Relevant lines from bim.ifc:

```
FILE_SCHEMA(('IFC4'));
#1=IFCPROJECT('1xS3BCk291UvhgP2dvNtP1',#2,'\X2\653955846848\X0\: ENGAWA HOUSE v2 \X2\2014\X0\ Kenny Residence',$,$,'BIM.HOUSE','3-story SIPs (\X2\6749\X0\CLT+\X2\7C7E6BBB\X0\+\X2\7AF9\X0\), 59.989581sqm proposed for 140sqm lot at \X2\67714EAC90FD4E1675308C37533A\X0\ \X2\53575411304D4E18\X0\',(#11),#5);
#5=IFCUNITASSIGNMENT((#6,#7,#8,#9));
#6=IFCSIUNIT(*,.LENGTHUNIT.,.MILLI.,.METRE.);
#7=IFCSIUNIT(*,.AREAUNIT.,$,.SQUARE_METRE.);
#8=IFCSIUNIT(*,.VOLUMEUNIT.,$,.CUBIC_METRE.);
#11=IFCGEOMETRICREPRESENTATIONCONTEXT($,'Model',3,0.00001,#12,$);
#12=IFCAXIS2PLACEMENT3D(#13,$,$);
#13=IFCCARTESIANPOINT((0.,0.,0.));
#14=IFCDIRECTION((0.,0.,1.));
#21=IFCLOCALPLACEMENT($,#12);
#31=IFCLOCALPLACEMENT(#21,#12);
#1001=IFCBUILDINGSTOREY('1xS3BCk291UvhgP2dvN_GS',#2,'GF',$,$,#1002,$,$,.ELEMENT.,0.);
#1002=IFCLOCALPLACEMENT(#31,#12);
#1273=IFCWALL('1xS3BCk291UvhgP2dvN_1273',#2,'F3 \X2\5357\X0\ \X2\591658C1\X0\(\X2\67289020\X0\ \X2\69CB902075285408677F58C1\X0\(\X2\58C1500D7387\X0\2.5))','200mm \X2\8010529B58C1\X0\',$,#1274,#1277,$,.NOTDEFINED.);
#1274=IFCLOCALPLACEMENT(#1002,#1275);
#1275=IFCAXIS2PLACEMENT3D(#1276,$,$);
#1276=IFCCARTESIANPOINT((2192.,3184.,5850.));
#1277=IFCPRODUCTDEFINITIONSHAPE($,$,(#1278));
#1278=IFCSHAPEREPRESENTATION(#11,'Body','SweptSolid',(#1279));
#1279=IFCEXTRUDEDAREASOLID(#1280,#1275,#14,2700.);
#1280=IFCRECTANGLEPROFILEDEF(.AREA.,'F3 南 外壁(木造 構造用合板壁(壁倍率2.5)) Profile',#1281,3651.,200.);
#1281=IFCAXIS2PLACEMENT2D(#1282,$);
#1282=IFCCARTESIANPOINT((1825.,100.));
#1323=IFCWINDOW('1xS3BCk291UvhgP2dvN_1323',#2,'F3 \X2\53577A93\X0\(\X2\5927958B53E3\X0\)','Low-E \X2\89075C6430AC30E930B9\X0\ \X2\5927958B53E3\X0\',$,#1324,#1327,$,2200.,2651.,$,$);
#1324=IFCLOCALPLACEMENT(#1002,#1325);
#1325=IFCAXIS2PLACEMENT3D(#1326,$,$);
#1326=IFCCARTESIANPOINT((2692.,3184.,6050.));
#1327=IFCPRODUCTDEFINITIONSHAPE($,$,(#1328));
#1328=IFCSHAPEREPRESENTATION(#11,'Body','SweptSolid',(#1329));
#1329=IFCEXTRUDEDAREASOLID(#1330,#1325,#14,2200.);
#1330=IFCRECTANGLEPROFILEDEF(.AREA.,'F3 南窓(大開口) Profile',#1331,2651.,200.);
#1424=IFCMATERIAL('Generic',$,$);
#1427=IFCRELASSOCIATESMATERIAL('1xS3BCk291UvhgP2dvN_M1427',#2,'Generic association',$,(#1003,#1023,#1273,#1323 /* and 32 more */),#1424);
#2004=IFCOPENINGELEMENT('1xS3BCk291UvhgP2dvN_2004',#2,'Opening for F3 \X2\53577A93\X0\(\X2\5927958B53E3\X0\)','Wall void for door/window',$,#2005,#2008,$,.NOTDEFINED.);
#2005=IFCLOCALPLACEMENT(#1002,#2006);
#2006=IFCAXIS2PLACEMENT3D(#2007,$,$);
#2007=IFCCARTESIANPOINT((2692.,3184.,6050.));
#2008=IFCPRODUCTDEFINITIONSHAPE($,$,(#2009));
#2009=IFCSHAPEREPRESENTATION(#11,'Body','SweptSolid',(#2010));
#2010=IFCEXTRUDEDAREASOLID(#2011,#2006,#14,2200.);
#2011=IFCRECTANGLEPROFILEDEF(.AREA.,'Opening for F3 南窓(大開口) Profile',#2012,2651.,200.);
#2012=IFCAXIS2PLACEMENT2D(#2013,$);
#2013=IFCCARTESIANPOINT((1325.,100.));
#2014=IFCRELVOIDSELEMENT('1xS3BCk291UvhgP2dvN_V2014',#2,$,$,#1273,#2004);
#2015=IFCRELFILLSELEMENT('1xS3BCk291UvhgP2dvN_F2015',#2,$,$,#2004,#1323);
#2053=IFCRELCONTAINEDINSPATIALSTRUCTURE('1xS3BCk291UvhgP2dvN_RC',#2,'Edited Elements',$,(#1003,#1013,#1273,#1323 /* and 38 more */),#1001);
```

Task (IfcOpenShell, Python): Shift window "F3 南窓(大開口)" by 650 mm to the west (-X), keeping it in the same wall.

```python
import ifcopenshell
import ifcopenshell.api.geometry
import ifcopenshell.util.placement

model = ifcopenshell.open("bim.ifc")

window = model.by_guid("1xS3BCk291UvhgP2dvN_1323")
opening = window.FillsVoids[0].RelatingOpeningElement
wall = opening.VoidsElements[0].RelatingBuildingElement

wall_matrix = ifcopenshell.util.placement.get_local_placement(wall.ObjectPlacement)
shift = wall_matrix[:3, 0] * -650.0
before = ifcopenshell.util.placement.get_local_placement(window.ObjectPlacement)[:3, 3].copy()

# The window is not placed relative to its opening, so move both.
for product in (opening, window):
    matrix = ifcopenshell.util.placement.get_local_placement(product.ObjectPlacement)
    matrix[:3, 3] += shift
    ifcopenshell.api.geometry.edit_object_placement(model, product=product, matrix=matrix, is_si=False)

after = ifcopenshell.util.placement.get_local_placement(window.ObjectPlacement)[:3, 3]
print("window moved by", (after - before).round(3) + 0.0)

model.write("bim-out.ifc")
```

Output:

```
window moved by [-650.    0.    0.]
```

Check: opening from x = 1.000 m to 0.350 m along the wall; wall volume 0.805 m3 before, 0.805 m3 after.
